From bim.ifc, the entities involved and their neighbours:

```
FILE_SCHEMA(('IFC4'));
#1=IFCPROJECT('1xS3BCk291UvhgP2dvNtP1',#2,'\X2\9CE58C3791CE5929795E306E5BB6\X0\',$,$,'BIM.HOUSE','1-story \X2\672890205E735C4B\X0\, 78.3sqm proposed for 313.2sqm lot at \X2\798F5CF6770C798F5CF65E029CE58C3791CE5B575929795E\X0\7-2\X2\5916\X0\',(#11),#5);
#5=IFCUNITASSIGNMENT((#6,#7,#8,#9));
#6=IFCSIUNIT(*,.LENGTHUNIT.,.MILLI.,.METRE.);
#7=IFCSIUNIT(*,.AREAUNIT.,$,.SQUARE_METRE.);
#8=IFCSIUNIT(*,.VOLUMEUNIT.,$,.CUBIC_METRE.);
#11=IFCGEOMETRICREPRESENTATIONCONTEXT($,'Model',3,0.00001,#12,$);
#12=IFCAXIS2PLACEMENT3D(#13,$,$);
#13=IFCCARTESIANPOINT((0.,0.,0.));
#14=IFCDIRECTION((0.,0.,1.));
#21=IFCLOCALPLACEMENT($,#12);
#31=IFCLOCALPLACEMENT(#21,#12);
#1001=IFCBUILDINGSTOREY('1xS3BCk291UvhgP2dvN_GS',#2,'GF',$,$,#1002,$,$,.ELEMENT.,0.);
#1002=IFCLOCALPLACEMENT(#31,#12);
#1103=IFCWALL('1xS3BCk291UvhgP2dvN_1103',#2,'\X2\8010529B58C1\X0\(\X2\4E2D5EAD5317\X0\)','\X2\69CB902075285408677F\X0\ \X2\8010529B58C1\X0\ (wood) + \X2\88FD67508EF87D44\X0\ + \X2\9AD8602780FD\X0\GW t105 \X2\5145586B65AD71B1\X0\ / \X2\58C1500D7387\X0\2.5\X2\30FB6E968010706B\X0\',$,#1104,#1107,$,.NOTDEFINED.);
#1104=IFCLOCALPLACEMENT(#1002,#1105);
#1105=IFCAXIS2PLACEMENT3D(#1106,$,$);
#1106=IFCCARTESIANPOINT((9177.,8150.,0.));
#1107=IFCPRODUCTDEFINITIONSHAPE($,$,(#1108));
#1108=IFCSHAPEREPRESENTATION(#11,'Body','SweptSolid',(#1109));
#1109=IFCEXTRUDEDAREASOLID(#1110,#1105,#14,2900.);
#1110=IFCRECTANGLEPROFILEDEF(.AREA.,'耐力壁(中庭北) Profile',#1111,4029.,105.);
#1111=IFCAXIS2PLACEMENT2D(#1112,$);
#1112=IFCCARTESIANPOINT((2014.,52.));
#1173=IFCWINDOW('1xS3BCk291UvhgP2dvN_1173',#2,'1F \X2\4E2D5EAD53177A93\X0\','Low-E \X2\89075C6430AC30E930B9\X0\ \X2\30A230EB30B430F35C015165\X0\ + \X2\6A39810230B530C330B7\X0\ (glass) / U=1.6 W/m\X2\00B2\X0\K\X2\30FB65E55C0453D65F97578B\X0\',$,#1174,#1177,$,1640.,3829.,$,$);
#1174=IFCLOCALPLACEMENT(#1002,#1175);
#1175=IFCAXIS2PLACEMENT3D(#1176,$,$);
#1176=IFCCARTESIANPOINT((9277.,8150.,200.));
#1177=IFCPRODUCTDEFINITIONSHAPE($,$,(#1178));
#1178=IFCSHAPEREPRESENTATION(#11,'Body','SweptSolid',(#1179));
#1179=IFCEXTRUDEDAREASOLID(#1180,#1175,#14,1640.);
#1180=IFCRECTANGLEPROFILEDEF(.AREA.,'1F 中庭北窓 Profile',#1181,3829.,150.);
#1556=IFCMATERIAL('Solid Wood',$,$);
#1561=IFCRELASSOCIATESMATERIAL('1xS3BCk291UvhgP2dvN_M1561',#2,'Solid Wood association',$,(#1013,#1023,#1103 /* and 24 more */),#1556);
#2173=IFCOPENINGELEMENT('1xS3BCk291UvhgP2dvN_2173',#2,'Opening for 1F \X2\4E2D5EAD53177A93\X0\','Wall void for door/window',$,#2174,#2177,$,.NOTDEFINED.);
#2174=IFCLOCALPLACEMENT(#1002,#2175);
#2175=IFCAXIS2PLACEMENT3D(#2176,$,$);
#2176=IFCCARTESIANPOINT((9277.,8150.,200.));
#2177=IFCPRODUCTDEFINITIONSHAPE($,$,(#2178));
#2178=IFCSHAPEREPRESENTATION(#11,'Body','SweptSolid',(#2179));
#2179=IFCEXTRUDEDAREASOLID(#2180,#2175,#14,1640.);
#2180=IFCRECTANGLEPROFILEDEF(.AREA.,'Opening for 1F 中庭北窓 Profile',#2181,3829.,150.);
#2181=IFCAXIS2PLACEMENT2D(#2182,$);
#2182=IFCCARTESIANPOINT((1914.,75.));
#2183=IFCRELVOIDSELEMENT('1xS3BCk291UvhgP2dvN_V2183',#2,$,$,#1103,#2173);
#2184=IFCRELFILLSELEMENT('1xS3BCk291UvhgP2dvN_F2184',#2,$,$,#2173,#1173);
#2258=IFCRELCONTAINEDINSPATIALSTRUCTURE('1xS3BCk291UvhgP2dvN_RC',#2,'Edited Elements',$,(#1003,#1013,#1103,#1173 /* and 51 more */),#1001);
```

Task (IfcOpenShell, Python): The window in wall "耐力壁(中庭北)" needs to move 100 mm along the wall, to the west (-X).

```python
import ifcopenshell
import ifcopenshell.api.geometry
import ifcopenshell.util.placement
import ifcopenshell.util.unit

model = ifcopenshell.open("bim.ifc")
unit_scale = ifcopenshell.util.unit.calculate_unit_scale(model)

window = model.by_guid("1xS3BCk291UvhgP2dvN_1173")
opening = window.FillsVoids[0].RelatingOpeningElement
wall = opening.VoidsElements[0].RelatingBuildingElement

wall_matrix = ifcopenshell.util.placement.get_local_placement(wall.ObjectPlacement)
shift = wall_matrix[:3, 0] * -0.1 / unit_scale
before = ifcopenshell.util.placement.get_local_placement(window.ObjectPlacement)[:3, 3].copy()

# The window is not placed relative to its opening, so move both.
for product in (opening, window):
    matrix = ifcopenshell.util.placement.get_local_placement(product.ObjectPlacement)
    matrix[:3, 3] += shift
    ifcopenshell.api.geometry.edit_object_placement(model, product=product, matrix=matrix, is_si=False)

after = ifcopenshell.util.placement.get_local_placement(window.ObjectPlacement)[:3, 3]
print("window moved by", (after - before).round(3) + 0.0)

model.write("bim_v2.ifc")
```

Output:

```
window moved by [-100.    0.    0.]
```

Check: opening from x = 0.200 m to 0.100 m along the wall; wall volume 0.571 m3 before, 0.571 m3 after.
